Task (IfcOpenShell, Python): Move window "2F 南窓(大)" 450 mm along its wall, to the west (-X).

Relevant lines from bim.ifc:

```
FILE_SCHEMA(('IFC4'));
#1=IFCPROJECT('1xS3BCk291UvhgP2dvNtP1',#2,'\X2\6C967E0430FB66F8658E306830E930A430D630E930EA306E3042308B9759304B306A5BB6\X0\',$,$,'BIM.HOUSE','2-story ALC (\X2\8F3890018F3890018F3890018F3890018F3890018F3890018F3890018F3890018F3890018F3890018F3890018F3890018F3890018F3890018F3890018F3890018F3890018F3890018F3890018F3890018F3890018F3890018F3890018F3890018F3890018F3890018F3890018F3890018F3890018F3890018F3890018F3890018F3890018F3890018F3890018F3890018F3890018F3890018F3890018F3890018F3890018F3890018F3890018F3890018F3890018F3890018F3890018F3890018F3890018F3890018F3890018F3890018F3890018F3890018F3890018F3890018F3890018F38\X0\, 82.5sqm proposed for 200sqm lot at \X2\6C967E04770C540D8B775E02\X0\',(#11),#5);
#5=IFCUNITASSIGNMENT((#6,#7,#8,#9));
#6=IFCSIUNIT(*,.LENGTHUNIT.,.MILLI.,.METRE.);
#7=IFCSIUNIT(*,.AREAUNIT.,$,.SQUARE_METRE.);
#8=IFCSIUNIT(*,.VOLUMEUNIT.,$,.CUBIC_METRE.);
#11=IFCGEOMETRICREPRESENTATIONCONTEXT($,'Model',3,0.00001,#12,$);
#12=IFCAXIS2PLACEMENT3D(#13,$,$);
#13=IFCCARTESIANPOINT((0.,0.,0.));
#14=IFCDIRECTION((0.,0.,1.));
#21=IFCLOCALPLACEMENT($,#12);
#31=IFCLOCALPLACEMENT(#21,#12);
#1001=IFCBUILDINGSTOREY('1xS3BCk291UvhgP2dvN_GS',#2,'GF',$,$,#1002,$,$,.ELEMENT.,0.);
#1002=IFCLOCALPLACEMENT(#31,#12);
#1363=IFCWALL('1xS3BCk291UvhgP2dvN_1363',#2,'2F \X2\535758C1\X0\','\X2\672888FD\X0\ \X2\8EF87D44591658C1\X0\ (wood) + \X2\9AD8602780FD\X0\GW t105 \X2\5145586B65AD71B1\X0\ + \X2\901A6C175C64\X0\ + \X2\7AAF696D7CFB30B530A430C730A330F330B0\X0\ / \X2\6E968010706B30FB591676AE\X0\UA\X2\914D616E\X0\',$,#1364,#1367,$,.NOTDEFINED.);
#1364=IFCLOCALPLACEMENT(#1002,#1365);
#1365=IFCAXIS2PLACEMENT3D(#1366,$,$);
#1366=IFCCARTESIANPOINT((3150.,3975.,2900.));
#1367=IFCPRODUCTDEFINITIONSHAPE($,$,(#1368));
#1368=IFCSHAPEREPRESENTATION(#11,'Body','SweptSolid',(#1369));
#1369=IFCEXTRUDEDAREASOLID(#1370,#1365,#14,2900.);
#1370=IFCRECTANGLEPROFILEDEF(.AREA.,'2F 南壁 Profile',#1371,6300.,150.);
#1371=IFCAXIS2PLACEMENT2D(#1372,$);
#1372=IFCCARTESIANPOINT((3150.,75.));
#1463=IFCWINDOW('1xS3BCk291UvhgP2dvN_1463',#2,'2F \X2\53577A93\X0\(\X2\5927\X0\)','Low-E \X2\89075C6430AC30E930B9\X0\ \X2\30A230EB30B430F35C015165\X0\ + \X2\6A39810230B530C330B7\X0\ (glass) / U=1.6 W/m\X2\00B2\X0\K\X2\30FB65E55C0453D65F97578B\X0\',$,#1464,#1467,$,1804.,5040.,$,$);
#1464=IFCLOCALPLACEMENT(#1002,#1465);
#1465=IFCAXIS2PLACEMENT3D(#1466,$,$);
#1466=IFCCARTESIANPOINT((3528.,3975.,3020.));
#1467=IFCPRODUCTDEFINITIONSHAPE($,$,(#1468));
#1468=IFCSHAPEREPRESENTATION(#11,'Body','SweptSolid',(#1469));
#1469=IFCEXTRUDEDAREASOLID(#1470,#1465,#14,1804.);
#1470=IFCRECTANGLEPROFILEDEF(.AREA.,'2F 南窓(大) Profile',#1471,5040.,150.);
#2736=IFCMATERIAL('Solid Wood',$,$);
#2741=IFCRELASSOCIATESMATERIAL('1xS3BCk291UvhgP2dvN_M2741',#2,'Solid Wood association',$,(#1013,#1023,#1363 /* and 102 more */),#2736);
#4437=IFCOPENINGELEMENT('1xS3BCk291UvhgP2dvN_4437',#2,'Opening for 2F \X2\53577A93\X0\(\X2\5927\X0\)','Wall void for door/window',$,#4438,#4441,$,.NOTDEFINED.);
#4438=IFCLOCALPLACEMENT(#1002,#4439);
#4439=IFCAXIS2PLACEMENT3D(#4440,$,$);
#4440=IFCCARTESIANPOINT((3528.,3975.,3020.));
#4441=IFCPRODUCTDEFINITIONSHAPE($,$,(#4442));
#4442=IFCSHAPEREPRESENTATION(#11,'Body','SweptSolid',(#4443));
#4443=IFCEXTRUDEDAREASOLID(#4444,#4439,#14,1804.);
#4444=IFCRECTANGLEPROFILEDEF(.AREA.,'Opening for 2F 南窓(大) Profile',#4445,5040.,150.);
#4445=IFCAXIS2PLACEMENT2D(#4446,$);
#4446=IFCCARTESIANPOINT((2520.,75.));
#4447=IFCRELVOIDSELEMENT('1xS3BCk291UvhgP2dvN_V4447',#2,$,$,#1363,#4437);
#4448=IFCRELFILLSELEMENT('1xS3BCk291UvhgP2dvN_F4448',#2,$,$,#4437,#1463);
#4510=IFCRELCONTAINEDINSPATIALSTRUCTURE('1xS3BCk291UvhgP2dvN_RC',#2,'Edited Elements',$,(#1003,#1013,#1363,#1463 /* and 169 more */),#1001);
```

```python
import ifcopenshell
import ifcopenshell.api.geometry
import ifcopenshell.util.placement
import ifcopenshell.util.unit

model = ifcopenshell.open("bim.ifc")
unit_scale = ifcopenshell.util.unit.calculate_unit_scale(model)

window = model.by_guid("1xS3BCk291UvhgP2dvN_1463")
opening = window.FillsVoids[0].RelatingOpeningElement
wall = opening.VoidsElements[0].RelatingBuildingElement

wall_matrix = ifcopenshell.util.placement.get_local_placement(wall.ObjectPlacement)
shift = wall_matrix[:3, 0] * -0.45 / unit_scale
before = ifcopenshell.util.placement.get_local_placement(window.ObjectPlacement)[:3, 3].copy()

# The window is not placed relative to its opening, so move both.
for product in (opening, window):
    matrix = ifcopenshell.util.placement.get_local_placement(product.ObjectPlacement)
    matrix[:3, 3] += shift
    ifcopenshell.api.geometry.edit_object_placement(model, product=product, matrix=matrix, is_si=False)

after = ifcopenshell.util.placement.get_local_placement(window.ObjectPlacement)[:3, 3]
print("window moved by", (after - before).round(3) + 0.0)

model.write("bim_updated.ifc")
```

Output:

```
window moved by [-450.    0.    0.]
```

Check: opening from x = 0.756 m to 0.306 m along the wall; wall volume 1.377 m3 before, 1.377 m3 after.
